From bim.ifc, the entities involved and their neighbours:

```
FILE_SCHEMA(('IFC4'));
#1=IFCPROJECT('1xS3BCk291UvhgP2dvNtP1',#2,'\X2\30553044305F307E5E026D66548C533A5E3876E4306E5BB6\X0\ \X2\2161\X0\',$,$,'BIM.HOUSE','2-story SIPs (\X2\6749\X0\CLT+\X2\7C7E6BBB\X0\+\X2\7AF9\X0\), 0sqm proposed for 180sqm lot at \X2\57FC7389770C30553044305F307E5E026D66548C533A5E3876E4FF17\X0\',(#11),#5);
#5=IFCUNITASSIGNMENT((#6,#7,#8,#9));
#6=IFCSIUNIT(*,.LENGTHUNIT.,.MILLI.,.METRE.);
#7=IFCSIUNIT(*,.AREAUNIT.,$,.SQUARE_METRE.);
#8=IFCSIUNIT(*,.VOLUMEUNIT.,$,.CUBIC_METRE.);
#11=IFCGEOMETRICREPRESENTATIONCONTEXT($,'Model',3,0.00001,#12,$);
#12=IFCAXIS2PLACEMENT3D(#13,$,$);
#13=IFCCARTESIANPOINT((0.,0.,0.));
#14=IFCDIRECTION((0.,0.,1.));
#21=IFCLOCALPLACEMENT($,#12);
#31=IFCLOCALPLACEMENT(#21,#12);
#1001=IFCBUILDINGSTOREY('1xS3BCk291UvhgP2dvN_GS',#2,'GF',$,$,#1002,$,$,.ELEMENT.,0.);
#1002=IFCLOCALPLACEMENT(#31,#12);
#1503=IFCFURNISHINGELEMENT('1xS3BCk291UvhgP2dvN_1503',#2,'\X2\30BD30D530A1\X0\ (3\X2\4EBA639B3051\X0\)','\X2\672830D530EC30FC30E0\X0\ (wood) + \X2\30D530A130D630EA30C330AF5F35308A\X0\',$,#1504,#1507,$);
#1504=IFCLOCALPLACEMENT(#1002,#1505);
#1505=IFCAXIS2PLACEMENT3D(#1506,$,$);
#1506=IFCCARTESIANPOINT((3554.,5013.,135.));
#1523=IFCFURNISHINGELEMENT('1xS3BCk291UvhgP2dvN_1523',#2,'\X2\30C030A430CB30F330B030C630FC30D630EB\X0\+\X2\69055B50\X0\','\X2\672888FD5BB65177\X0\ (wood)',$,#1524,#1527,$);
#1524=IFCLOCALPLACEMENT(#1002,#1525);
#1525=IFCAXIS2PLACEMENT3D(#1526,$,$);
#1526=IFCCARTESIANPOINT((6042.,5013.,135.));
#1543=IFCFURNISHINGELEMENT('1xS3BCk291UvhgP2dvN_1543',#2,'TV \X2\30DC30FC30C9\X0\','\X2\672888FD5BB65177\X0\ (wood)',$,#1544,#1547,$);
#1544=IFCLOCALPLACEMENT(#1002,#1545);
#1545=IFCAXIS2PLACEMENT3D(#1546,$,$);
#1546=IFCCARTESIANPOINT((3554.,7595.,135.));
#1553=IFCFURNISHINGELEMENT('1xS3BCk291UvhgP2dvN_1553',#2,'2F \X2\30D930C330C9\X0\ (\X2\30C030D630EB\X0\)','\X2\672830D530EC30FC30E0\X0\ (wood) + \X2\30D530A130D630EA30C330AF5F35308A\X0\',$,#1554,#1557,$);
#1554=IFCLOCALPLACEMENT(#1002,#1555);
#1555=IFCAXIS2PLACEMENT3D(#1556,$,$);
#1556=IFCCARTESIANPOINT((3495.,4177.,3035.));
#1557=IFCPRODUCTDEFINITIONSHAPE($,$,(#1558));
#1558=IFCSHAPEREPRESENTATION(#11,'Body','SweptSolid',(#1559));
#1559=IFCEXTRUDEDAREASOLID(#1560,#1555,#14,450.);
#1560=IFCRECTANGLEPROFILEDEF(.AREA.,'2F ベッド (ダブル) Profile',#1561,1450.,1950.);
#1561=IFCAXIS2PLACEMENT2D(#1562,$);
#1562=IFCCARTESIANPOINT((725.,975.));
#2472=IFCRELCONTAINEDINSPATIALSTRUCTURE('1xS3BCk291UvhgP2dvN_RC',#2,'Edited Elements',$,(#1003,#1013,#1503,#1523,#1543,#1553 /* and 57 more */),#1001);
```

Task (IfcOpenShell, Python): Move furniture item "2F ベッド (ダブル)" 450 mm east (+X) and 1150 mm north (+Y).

```python
import ifcopenshell
import ifcopenshell.api.geometry
import ifcopenshell.util.placement

model = ifcopenshell.open("bim.ifc")

item = model.by_guid("1xS3BCk291UvhgP2dvN_1553")
matrix = ifcopenshell.util.placement.get_local_placement(item.ObjectPlacement)
matrix[0, 3] += 450.0
matrix[1, 3] += 1150.0
ifcopenshell.api.geometry.edit_object_placement(model, product=item, matrix=matrix, is_si=False)

print(ifcopenshell.util.placement.get_local_placement(item.ObjectPlacement).round(3) + 0.0)

model.write("bim_edited.ifc")
```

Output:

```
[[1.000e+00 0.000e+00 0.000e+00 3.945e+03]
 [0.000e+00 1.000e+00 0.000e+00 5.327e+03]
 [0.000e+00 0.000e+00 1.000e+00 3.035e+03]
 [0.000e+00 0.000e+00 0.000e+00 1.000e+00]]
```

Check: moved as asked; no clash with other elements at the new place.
